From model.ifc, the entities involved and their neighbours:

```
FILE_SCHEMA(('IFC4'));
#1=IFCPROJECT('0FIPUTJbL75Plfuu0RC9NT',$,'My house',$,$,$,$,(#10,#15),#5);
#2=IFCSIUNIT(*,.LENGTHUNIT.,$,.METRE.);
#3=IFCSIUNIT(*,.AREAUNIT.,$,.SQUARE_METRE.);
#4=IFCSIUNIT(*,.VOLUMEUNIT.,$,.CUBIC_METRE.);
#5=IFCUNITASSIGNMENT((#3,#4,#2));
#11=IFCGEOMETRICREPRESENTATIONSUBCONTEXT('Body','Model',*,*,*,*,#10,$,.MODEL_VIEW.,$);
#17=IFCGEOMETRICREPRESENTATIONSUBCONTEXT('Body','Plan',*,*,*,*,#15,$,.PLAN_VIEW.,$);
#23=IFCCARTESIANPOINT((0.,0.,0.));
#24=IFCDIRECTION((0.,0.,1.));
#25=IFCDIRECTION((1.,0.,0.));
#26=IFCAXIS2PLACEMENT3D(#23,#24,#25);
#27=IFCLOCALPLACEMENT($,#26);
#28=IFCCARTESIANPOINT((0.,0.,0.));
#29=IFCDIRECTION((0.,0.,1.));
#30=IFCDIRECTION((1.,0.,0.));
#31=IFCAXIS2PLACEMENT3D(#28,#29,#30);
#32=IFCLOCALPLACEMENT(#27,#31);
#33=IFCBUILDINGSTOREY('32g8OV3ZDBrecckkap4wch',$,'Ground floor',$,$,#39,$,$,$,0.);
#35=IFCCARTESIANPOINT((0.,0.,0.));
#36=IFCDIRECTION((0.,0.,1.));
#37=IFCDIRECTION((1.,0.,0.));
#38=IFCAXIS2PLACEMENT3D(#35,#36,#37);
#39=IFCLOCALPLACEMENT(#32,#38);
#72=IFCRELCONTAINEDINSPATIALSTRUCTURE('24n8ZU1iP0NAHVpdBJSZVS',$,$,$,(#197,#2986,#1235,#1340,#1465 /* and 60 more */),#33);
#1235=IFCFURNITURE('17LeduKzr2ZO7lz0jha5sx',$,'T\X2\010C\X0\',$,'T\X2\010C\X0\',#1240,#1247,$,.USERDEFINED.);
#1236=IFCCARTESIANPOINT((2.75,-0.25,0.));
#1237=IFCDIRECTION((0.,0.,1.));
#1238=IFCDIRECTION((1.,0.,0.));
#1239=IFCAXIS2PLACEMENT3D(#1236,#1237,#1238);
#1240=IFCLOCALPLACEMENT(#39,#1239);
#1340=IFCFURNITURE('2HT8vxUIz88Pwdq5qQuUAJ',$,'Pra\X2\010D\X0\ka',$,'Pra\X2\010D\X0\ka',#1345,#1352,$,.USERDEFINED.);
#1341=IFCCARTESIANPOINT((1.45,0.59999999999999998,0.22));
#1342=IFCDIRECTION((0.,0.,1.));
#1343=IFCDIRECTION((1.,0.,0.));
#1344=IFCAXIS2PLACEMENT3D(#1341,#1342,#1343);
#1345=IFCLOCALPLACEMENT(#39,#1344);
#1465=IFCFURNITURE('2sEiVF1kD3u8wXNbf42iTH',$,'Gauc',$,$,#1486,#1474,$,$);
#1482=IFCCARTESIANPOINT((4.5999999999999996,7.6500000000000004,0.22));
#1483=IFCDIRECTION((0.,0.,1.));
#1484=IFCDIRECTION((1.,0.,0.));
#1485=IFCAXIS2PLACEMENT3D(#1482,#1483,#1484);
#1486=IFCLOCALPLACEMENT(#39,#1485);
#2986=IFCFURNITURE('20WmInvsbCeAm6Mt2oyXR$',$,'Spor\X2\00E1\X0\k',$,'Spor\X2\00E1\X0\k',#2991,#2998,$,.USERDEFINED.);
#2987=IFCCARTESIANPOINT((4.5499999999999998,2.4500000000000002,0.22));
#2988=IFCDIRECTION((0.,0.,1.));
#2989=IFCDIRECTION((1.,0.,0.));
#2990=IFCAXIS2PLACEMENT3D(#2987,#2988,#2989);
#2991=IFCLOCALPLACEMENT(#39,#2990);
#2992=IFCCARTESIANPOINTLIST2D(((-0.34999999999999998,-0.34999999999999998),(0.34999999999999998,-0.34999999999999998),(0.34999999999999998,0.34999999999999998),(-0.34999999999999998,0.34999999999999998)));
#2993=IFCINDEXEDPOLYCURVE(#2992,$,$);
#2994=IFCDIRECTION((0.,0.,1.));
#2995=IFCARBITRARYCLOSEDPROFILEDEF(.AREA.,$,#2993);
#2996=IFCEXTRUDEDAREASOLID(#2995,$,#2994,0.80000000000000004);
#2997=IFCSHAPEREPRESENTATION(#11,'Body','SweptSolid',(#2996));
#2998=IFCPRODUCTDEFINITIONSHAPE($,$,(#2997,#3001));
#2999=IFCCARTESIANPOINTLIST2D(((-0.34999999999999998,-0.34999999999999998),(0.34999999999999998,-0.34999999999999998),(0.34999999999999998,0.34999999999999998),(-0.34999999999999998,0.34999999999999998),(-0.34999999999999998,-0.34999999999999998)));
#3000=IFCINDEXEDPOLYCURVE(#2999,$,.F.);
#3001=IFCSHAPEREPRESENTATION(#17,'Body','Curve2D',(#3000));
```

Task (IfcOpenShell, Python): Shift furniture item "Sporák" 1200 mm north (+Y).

```python
import ifcopenshell
import ifcopenshell.api.geometry
import ifcopenshell.util.placement
import ifcopenshell.util.unit

model = ifcopenshell.open("model.ifc")
unit_scale = ifcopenshell.util.unit.calculate_unit_scale(model)

item = model.by_guid("20WmInvsbCeAm6Mt2oyXR$")
matrix = ifcopenshell.util.placement.get_local_placement(item.ObjectPlacement)
matrix[1, 3] += 1.2 / unit_scale
ifcopenshell.api.geometry.edit_object_placement(model, product=item, matrix=matrix, is_si=False)

print(ifcopenshell.util.placement.get_local_placement(item.ObjectPlacement).round(3) + 0.0)

model.write("model_v2.ifc")
```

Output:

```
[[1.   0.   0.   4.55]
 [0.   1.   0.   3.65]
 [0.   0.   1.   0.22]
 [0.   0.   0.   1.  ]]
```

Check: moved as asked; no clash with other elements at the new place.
